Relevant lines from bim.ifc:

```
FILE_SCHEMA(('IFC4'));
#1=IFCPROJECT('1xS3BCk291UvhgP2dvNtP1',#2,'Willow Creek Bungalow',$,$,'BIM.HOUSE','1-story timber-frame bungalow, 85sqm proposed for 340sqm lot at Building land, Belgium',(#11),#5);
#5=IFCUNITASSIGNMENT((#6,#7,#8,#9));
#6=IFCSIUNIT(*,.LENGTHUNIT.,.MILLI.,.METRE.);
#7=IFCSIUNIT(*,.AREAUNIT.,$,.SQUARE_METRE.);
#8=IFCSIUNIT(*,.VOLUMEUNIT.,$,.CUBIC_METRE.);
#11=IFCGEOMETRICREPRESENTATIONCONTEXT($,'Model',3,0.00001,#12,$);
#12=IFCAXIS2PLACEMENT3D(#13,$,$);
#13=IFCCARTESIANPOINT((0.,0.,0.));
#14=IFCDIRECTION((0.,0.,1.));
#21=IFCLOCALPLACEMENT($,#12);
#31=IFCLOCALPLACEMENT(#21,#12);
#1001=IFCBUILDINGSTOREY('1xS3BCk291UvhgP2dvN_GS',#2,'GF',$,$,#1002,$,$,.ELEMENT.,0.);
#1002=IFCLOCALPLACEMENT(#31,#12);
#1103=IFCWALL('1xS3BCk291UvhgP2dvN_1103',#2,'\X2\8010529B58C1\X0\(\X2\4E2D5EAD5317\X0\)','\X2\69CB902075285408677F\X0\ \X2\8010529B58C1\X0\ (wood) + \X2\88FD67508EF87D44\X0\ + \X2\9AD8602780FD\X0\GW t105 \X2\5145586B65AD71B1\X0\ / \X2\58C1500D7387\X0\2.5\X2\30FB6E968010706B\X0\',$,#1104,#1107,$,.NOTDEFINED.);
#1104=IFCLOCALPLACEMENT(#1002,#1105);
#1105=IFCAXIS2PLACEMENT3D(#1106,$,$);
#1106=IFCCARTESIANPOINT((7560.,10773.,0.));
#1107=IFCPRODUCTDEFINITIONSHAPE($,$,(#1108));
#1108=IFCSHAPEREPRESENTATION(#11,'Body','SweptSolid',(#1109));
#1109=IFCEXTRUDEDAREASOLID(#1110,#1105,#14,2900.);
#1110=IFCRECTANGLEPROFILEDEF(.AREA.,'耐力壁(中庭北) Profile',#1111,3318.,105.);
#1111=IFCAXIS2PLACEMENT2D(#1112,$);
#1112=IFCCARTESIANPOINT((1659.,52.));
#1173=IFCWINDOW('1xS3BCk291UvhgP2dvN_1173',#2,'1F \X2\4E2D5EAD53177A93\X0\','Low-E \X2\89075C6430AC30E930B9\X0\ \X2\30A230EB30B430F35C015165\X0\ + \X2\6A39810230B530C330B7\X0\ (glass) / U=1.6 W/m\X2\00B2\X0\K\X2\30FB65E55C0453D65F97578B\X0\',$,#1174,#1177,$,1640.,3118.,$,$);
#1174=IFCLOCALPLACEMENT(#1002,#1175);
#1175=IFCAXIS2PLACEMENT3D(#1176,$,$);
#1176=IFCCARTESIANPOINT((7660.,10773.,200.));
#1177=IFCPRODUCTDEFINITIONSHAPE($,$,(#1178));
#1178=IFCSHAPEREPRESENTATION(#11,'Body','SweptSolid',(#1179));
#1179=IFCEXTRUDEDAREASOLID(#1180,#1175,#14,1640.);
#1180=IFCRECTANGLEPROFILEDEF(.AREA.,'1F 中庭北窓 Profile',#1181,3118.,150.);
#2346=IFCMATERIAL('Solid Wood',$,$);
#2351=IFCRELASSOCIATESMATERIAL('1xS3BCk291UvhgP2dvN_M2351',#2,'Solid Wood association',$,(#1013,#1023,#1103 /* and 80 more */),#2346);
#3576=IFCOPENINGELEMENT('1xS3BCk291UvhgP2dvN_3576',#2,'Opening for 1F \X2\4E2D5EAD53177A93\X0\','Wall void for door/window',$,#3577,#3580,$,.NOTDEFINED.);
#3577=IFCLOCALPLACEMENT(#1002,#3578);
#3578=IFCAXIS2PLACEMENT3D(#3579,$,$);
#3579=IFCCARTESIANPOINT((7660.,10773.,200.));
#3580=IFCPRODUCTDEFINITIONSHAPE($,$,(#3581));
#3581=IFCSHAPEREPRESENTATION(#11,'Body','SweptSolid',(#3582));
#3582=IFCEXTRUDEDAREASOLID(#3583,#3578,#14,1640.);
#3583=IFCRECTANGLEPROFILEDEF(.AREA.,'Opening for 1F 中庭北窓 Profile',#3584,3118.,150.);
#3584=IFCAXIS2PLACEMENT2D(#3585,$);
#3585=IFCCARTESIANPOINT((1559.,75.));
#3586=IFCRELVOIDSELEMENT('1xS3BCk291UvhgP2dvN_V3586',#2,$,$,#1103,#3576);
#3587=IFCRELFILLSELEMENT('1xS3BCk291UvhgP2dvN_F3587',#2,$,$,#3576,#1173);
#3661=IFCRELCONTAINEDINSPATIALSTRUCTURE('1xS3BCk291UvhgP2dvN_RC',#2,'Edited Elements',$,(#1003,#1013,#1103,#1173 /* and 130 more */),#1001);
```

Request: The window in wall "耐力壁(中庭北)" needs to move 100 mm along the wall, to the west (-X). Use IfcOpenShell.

```python
import ifcopenshell
import ifcopenshell.api.geometry
import ifcopenshell.util.placement
import ifcopenshell.util.unit

model = ifcopenshell.open("bim.ifc")
unit_scale = ifcopenshell.util.unit.calculate_unit_scale(model)

window = model.by_guid("1xS3BCk291UvhgP2dvN_1173")
opening = window.FillsVoids[0].RelatingOpeningElement
wall = opening.VoidsElements[0].RelatingBuildingElement

wall_matrix = ifcopenshell.util.placement.get_local_placement(wall.ObjectPlacement)
shift = wall_matrix[:3, 0] * -0.1 / unit_scale
before = ifcopenshell.util.placement.get_local_placement(window.ObjectPlacement)[:3, 3].copy()

# The window is not placed relative to its opening, so move both.
for product in (opening, window):
    matrix = ifcopenshell.util.placement.get_local_placement(product.ObjectPlacement)
    matrix[:3, 3] += shift
    ifcopenshell.api.geometry.edit_object_placement(model, product=product, matrix=matrix, is_si=False)

after = ifcopenshell.util.placement.get_local_placement(window.ObjectPlacement)[:3, 3]
print("window moved by", (after - before).round(3) + 0.0)

model.write("bim-out.ifc")
```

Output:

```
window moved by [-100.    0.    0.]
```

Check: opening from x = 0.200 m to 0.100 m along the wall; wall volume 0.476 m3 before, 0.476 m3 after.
